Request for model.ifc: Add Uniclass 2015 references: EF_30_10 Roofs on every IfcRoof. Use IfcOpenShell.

First a look at what the model holds.

```python
import ifcopenshell

model = ifcopenshell.open("model.ifc")
print(model.schema)
print("classifications:", [c.Name for c in model.by_type("IfcClassification")])
for ifc_class in ("IfcDoor", "IfcRoof", "IfcStair", "IfcWall", "IfcWindow"):
    print(ifc_class, len(model.by_type(ifc_class)))
```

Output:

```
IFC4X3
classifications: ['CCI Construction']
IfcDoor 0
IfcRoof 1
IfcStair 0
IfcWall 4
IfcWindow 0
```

```python
import ifcopenshell
import ifcopenshell.api.classification

model = ifcopenshell.open("model.ifc")

system = ifcopenshell.api.classification.add_classification(model, classification="Uniclass 2015")

codes = {
    "IfcRoof": ("EF_30_10", "Roofs"),
}
for ifc_class, (code, name) in codes.items():
    products = model.by_type(ifc_class)
    ifcopenshell.api.classification.add_reference(
        model, products=products, classification=system, identification=code, name=name
    )
    print(code, len(products))

model.write("model_v2.ifc")
```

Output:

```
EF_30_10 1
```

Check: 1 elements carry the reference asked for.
